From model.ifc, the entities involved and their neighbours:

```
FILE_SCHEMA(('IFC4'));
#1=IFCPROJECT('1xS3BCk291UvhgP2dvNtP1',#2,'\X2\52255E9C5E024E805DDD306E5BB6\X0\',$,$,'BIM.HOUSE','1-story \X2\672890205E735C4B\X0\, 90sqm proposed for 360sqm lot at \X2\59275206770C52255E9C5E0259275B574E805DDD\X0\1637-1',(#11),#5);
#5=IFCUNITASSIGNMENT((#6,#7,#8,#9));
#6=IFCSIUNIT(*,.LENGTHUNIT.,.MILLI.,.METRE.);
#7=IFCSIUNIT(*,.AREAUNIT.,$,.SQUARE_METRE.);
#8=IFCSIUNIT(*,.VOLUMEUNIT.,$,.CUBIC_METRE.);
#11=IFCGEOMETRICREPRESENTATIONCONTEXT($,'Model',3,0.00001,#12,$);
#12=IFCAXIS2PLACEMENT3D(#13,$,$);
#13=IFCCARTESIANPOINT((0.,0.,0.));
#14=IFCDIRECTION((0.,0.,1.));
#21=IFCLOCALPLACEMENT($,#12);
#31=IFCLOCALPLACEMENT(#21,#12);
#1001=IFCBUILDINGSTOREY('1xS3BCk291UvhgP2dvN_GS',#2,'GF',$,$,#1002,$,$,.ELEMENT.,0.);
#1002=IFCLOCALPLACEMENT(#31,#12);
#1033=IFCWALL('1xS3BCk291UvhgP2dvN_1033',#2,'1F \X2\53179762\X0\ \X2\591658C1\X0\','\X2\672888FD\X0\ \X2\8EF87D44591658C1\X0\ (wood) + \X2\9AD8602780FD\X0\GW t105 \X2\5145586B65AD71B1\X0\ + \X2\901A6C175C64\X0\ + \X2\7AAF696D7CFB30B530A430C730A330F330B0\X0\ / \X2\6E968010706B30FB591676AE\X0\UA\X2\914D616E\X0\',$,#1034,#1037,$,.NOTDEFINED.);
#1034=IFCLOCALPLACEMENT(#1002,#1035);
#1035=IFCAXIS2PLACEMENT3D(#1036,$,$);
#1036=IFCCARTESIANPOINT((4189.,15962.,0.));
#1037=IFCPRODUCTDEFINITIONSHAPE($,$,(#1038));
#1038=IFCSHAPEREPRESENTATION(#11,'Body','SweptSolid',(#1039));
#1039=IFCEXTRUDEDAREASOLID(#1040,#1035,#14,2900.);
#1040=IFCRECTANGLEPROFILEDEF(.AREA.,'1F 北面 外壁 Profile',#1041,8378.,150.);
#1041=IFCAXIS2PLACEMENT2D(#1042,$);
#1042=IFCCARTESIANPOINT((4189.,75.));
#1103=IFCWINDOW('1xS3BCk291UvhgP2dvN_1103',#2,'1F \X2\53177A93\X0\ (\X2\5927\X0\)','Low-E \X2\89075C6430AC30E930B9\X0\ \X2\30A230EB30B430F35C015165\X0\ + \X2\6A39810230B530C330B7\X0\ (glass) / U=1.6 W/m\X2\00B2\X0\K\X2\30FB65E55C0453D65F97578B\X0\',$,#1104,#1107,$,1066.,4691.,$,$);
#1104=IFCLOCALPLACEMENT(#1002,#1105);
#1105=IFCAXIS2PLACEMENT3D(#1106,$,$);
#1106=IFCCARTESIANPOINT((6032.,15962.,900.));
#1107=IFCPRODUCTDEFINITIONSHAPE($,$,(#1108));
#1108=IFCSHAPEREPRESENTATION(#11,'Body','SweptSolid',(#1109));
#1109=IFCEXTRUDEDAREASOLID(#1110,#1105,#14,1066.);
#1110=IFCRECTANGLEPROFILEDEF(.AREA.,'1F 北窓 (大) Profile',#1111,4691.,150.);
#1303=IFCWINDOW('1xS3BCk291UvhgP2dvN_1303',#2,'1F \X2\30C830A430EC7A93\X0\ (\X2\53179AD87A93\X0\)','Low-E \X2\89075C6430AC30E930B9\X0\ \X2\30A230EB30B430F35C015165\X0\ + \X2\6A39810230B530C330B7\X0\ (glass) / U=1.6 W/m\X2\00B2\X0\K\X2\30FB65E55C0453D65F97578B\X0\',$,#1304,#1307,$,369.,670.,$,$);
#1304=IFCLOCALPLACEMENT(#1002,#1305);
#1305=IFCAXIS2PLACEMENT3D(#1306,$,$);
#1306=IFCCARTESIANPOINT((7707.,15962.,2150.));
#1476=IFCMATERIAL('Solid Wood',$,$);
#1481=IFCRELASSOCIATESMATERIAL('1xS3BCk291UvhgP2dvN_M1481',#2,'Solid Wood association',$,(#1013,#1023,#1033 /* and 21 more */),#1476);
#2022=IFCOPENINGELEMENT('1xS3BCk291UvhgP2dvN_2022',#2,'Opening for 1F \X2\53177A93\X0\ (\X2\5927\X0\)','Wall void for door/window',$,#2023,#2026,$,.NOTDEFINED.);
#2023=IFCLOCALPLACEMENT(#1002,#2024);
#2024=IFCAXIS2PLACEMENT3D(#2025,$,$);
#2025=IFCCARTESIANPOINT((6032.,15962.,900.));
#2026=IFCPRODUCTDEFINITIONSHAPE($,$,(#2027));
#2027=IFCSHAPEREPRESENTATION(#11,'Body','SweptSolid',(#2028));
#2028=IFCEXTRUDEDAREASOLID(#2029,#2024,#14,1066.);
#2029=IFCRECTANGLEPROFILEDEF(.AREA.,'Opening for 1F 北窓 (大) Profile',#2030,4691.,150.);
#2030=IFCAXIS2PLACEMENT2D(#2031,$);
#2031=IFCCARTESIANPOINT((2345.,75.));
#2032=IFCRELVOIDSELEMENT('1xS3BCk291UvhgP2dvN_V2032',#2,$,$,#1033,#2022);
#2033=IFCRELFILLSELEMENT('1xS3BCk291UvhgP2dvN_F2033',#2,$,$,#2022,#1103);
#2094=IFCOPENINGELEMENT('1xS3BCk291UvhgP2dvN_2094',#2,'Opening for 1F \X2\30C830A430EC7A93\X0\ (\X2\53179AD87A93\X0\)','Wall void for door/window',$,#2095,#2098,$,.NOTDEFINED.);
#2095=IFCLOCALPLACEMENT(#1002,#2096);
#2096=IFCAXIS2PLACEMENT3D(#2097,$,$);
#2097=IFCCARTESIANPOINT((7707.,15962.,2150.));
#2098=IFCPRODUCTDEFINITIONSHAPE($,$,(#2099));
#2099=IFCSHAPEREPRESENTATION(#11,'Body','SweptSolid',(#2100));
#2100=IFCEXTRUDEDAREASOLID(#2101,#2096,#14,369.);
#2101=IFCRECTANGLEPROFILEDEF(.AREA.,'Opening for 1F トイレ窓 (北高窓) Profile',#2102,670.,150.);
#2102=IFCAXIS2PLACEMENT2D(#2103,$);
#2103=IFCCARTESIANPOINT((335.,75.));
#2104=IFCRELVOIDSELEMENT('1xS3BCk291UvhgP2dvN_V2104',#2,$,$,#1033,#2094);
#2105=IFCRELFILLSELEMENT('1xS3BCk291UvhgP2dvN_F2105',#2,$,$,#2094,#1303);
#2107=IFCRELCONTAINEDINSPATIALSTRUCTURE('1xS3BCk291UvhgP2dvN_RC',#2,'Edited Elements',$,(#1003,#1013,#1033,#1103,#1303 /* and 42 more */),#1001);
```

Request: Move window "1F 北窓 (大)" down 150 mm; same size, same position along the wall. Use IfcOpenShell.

```python
import numpy as np
import ifcopenshell
import ifcopenshell.api.geometry
import ifcopenshell.util.placement
import ifcopenshell.util.unit

model = ifcopenshell.open("model.ifc")
unit_scale = ifcopenshell.util.unit.calculate_unit_scale(model)

window = model.by_guid("1xS3BCk291UvhgP2dvN_1103")
opening = window.FillsVoids[0].RelatingOpeningElement
dz = -0.15 / unit_scale

shift = np.array([0.0, 0.0, dz])
# The window is not placed relative to its opening, so move both.
for product in (opening, window):
    matrix = ifcopenshell.util.placement.get_local_placement(product.ObjectPlacement)
    matrix[:3, 3] += shift
    ifcopenshell.api.geometry.edit_object_placement(model, product=product, matrix=matrix, is_si=False)

print(f"moved by {dz * unit_scale:+.3f} m")

model.write("model_updated.ifc")
```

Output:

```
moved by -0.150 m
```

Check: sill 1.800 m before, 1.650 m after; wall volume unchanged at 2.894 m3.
